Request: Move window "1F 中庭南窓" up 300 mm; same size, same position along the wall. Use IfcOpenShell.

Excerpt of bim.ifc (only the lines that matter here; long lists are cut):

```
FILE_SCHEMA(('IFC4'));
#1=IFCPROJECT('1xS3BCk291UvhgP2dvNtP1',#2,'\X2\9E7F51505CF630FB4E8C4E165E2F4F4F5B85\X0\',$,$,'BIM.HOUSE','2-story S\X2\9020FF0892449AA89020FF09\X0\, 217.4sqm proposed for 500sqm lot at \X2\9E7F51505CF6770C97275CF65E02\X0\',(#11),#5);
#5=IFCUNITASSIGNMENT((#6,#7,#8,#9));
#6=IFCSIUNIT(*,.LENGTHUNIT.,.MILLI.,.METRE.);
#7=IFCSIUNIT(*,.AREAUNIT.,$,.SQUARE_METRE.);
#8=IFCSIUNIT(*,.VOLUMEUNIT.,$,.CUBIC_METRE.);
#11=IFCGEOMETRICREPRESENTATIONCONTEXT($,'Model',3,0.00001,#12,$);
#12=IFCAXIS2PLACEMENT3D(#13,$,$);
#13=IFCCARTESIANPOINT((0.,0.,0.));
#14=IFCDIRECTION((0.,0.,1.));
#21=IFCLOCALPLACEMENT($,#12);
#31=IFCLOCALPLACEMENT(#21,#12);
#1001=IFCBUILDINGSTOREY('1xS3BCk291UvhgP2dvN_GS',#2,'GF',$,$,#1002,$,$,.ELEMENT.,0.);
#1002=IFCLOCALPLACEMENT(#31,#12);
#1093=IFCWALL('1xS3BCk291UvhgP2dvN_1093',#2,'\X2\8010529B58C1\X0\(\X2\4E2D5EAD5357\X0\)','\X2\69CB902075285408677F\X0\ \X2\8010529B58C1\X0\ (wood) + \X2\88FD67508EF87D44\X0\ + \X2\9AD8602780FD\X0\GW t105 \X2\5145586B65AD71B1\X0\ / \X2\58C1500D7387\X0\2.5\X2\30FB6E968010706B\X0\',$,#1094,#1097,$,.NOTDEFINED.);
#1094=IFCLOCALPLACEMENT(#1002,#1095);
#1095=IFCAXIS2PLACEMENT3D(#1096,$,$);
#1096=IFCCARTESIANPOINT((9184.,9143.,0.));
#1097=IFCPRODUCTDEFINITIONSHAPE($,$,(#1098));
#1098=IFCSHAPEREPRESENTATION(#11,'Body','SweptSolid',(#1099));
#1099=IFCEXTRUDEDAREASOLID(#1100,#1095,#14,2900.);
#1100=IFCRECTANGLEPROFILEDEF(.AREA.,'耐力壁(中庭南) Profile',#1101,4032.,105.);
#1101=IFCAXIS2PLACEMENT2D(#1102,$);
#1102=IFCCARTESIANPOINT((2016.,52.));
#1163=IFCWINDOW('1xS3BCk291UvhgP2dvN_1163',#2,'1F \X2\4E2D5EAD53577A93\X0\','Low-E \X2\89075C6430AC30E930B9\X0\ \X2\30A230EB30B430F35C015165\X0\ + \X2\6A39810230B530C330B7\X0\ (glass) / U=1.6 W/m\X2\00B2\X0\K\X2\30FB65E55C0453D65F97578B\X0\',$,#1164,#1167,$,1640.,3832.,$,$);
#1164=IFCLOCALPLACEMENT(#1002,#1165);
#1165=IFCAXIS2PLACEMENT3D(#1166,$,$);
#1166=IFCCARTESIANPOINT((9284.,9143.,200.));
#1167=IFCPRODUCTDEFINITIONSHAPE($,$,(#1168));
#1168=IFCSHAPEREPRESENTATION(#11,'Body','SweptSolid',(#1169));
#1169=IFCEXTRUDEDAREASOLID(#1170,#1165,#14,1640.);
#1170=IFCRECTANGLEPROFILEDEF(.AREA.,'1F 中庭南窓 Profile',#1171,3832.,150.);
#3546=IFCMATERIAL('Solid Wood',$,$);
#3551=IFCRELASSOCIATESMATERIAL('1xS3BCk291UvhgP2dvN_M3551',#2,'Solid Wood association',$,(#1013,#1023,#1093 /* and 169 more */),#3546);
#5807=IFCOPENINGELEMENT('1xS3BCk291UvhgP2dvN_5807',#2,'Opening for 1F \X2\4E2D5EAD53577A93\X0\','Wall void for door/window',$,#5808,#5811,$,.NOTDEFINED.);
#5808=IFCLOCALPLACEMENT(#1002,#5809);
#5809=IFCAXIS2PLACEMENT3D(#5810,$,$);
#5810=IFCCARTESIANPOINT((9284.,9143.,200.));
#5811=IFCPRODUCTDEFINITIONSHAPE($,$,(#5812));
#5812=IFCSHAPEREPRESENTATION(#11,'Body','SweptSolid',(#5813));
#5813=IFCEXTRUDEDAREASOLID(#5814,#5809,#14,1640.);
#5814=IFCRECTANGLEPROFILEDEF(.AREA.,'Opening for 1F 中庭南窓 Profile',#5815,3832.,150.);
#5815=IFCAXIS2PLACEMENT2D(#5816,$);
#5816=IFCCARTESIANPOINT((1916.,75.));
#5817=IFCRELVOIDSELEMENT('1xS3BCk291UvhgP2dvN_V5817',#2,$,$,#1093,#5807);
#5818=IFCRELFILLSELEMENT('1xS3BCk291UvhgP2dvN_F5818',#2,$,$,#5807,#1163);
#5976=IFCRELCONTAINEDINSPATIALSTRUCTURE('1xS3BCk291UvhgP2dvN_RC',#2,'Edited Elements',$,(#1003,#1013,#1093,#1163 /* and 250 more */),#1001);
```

```python
import numpy as np
import ifcopenshell
import ifcopenshell.api.geometry
import ifcopenshell.util.placement
import ifcopenshell.util.unit

model = ifcopenshell.open("bim.ifc")
unit_scale = ifcopenshell.util.unit.calculate_unit_scale(model)

window = model.by_guid("1xS3BCk291UvhgP2dvN_1163")
opening = window.FillsVoids[0].RelatingOpeningElement
dz = 0.3 / unit_scale

shift = np.array([0.0, 0.0, dz])
# The window is not placed relative to its opening, so move both.
for product in (opening, window):
    matrix = ifcopenshell.util.placement.get_local_placement(product.ObjectPlacement)
    matrix[:3, 3] += shift
    ifcopenshell.api.geometry.edit_object_placement(model, product=product, matrix=matrix, is_si=False)

print(f"moved by {dz * unit_scale:+.3f} m")

model.write("bim_updated.ifc")
```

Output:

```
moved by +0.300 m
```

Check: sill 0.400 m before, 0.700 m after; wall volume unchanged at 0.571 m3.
